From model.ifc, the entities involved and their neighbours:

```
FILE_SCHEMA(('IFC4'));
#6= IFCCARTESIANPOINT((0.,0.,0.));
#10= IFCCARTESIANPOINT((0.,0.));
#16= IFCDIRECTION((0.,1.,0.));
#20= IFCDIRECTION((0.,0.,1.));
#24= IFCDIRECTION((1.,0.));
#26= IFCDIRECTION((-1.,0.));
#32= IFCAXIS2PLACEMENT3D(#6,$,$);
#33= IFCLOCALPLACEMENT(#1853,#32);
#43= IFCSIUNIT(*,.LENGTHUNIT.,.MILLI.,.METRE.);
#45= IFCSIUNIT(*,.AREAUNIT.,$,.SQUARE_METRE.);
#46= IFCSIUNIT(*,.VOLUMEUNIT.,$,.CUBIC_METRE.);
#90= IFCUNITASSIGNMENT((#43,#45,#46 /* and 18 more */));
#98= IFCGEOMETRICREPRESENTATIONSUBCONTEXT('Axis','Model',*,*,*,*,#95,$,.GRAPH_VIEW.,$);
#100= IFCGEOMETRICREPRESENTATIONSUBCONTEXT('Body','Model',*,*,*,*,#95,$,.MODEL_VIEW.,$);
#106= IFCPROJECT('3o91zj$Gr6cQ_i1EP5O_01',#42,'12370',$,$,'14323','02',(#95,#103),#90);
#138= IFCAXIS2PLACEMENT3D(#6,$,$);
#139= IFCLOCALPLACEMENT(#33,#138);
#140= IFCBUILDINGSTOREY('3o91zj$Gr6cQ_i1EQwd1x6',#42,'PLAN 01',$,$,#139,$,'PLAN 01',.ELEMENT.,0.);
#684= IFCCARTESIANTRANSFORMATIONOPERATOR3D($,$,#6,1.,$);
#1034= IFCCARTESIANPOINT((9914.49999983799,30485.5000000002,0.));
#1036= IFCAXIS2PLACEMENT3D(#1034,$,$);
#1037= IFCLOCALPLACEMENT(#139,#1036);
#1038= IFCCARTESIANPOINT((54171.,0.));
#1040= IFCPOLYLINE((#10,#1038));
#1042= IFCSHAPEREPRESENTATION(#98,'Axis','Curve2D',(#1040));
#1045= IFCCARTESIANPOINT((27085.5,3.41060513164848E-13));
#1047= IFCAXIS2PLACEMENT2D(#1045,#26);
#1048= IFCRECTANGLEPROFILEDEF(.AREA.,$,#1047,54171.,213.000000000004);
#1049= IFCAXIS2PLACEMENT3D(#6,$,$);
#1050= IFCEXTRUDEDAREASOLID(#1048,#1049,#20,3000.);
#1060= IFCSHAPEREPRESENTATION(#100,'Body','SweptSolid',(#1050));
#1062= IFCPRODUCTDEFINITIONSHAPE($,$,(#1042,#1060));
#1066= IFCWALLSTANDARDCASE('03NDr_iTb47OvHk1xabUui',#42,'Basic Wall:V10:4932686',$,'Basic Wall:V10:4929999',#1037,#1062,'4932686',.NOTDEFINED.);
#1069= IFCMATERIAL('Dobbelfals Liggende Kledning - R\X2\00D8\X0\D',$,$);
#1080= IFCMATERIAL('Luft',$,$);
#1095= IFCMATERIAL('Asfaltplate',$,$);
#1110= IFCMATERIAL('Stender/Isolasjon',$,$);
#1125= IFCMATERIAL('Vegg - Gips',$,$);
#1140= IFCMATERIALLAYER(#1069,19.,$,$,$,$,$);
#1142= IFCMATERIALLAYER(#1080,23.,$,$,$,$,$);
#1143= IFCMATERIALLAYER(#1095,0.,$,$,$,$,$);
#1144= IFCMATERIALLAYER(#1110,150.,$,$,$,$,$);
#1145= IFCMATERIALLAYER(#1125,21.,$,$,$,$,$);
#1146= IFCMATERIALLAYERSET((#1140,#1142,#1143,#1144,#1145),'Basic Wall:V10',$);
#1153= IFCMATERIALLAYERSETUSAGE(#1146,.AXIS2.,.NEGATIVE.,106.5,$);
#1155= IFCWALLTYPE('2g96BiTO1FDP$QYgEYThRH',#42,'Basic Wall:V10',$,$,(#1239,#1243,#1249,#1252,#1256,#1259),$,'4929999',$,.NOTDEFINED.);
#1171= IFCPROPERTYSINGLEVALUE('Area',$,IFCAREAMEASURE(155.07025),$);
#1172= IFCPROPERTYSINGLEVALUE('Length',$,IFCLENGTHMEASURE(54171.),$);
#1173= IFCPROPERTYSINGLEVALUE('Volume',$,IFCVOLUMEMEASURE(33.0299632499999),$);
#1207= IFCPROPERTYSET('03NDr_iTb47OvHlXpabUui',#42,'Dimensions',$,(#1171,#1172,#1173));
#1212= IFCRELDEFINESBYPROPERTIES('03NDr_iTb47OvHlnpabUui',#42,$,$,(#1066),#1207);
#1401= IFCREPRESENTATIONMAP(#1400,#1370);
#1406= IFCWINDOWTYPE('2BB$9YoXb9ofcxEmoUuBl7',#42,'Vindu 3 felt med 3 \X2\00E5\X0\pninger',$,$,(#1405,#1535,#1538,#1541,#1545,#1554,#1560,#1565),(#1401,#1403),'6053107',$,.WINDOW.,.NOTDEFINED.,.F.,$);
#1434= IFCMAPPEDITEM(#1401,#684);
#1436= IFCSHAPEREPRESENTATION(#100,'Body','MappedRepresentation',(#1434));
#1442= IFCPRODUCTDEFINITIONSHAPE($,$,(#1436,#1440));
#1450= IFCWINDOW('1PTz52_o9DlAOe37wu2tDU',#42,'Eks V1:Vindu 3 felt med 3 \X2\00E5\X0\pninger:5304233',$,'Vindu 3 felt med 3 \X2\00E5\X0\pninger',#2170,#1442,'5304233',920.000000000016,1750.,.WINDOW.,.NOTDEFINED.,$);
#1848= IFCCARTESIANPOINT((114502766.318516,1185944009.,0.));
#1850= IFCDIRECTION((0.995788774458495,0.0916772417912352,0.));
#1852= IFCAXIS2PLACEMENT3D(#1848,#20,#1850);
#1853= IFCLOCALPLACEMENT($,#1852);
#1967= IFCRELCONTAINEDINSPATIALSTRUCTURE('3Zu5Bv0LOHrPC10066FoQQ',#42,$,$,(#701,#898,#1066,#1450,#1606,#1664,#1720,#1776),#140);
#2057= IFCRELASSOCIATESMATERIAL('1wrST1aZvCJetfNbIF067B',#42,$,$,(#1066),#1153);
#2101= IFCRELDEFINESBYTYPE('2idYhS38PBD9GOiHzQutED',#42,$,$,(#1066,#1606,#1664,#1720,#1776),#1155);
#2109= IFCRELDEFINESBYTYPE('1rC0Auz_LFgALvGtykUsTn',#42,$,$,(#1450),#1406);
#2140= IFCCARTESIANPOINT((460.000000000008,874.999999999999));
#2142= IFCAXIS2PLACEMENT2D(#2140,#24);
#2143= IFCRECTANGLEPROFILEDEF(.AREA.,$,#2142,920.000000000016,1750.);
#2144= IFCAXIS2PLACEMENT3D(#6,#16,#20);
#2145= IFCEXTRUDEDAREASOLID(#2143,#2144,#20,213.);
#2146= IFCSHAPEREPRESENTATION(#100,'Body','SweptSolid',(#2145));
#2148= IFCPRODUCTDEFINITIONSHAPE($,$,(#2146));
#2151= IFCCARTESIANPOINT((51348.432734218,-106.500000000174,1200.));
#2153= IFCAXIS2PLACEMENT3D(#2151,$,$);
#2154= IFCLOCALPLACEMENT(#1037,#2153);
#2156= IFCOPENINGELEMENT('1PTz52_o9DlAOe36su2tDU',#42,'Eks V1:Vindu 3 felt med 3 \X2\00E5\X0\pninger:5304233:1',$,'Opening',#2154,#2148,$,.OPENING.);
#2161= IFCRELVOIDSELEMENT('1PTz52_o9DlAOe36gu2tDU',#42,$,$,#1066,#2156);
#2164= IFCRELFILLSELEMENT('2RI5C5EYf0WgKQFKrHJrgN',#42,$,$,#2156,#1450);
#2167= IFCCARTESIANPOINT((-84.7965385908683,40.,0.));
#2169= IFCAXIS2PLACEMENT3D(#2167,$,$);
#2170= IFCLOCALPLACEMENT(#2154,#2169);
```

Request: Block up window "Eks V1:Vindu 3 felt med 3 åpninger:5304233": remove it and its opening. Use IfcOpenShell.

```python
import ifcopenshell
import ifcopenshell.api.feature
import ifcopenshell.api.pset
import ifcopenshell.api.root
import ifcopenshell.geom
import ifcopenshell.util.element
import ifcopenshell.util.shape
import ifcopenshell.util.unit

model = ifcopenshell.open("model.ifc")
area_scale = ifcopenshell.util.unit.calculate_unit_scale(model, "AREAUNIT")
volume_scale = ifcopenshell.util.unit.calculate_unit_scale(model, "VOLUMEUNIT")
settings = ifcopenshell.geom.settings()


def volume(element):
    """Net volume in cubic metres, openings subtracted."""
    shape = ifcopenshell.geom.create_shape(settings, element)
    return ifcopenshell.util.shape.get_volume(shape.geometry)


window = model.by_guid("1PTz52_o9DlAOe37wu2tDU")
opening = window.FillsVoids[0].RelatingOpeningElement
wall = opening.VoidsElements[0].RelatingBuildingElement
before = volume(wall)

ifcopenshell.api.root.remove_product(model, product=window)
ifcopenshell.api.feature.remove_feature(model, feature=opening)

after = volume(wall)
thickness = 0.213  # wall thickness in metres

# Update the wall's stored quantities.
pset = model.by_id(ifcopenshell.util.element.get_pset(wall, "Dimensions", should_inherit=False)["id"])
ifcopenshell.api.pset.edit_pset(model, pset=pset, properties={
    "Area": model.create_entity("IfcAreaMeasure", after / thickness / area_scale),
    "Volume": model.create_entity("IfcVolumeMeasure", after / volume_scale),
})

print(f"wall volume {before:.3f} -> {after:.3f} m3")

model.write("model_v2.ifc")
```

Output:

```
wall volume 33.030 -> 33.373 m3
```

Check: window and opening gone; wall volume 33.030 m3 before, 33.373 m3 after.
